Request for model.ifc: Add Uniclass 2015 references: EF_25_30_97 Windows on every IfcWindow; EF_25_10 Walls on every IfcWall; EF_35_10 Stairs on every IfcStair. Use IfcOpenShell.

First a look at what the model holds.

```python
import ifcopenshell

model = ifcopenshell.open("model.ifc")
print(model.schema)
print("classifications:", [c.Name for c in model.by_type("IfcClassification")])
for ifc_class in ("IfcDoor", "IfcRoof", "IfcStair", "IfcWall", "IfcWindow"):
    print(ifc_class, len(model.by_type(ifc_class)))
```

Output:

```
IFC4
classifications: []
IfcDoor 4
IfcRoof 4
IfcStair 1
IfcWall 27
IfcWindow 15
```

```python
import ifcopenshell
import ifcopenshell.api.classification

model = ifcopenshell.open("model.ifc")

system = ifcopenshell.api.classification.add_classification(model, classification="Uniclass 2015")

codes = {
    "IfcWindow": ("EF_25_30_97", "Windows"),
    "IfcWall": ("EF_25_10", "Walls"),
    "IfcStair": ("EF_35_10", "Stairs"),
}
for ifc_class, (code, name) in codes.items():
    products = model.by_type(ifc_class)
    ifcopenshell.api.classification.add_reference(
        model, products=products, classification=system, identification=code, name=name
    )
    print(code, len(products))

model.write("model-out.ifc")
```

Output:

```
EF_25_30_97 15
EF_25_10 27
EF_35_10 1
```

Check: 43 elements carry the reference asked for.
